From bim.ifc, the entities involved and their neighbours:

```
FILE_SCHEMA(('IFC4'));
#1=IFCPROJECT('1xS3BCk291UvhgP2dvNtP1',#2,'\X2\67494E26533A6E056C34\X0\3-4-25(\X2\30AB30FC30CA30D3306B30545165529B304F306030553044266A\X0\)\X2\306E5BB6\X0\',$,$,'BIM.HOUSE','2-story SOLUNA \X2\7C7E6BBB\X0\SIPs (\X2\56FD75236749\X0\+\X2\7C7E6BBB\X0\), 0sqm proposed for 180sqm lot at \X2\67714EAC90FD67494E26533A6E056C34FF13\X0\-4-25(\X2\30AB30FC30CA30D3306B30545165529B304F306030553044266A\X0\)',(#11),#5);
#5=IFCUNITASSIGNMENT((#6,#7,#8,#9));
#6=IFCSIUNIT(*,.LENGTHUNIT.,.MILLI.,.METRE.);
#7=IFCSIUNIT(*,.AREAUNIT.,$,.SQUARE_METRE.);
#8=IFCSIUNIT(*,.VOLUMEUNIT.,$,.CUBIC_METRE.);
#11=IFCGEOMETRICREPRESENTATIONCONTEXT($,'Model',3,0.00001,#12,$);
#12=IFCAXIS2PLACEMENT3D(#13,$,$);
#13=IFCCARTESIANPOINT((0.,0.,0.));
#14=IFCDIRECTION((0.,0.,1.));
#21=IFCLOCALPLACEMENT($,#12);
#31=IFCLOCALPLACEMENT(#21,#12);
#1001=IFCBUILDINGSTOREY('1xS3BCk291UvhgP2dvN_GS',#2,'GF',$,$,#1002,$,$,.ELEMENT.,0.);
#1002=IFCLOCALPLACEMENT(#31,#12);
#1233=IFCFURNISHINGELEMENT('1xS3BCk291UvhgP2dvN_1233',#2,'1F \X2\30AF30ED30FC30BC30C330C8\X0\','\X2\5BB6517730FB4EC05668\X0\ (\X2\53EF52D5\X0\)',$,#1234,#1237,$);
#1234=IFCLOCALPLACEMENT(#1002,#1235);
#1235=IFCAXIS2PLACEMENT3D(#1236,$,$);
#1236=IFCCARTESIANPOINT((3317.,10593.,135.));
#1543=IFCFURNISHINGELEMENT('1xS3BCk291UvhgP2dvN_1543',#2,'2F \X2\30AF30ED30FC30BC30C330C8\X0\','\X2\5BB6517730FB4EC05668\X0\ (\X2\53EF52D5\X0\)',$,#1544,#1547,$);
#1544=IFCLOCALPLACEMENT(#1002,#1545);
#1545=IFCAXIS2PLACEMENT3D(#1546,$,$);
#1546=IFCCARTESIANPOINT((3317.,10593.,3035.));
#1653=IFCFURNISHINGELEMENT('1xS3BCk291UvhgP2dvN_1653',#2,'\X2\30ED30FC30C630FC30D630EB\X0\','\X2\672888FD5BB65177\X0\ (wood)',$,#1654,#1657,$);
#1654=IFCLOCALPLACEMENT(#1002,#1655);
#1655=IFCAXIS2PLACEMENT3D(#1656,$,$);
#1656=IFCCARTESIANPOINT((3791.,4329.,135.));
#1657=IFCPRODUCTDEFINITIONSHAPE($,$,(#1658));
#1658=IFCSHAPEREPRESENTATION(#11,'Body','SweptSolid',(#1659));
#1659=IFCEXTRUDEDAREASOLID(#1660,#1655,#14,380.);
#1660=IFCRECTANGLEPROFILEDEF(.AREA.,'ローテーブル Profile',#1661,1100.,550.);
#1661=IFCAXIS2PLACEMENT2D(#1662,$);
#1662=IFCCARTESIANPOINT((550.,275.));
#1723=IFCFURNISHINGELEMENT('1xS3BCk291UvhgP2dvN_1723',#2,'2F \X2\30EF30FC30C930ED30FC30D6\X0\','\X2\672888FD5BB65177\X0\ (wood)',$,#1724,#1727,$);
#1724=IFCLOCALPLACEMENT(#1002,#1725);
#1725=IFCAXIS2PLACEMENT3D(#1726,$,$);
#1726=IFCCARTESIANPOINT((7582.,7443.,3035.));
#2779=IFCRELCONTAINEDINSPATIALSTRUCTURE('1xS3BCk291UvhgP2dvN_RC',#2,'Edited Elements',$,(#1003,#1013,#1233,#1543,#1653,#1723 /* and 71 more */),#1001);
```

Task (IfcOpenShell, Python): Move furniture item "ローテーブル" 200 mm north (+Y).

```python
import ifcopenshell
import ifcopenshell.api.geometry
import ifcopenshell.util.placement
import ifcopenshell.util.unit

model = ifcopenshell.open("bim.ifc")
unit_scale = ifcopenshell.util.unit.calculate_unit_scale(model)

item = model.by_guid("1xS3BCk291UvhgP2dvN_1653")
matrix = ifcopenshell.util.placement.get_local_placement(item.ObjectPlacement)
matrix[1, 3] += 0.2 / unit_scale
ifcopenshell.api.geometry.edit_object_placement(model, product=item, matrix=matrix, is_si=False)

print(ifcopenshell.util.placement.get_local_placement(item.ObjectPlacement).round(3) + 0.0)

model.write("bim_rev.ifc")
```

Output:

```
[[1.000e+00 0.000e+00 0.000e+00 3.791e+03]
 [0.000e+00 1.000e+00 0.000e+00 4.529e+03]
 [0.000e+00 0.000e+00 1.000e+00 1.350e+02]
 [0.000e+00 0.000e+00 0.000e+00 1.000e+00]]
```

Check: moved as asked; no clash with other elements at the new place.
